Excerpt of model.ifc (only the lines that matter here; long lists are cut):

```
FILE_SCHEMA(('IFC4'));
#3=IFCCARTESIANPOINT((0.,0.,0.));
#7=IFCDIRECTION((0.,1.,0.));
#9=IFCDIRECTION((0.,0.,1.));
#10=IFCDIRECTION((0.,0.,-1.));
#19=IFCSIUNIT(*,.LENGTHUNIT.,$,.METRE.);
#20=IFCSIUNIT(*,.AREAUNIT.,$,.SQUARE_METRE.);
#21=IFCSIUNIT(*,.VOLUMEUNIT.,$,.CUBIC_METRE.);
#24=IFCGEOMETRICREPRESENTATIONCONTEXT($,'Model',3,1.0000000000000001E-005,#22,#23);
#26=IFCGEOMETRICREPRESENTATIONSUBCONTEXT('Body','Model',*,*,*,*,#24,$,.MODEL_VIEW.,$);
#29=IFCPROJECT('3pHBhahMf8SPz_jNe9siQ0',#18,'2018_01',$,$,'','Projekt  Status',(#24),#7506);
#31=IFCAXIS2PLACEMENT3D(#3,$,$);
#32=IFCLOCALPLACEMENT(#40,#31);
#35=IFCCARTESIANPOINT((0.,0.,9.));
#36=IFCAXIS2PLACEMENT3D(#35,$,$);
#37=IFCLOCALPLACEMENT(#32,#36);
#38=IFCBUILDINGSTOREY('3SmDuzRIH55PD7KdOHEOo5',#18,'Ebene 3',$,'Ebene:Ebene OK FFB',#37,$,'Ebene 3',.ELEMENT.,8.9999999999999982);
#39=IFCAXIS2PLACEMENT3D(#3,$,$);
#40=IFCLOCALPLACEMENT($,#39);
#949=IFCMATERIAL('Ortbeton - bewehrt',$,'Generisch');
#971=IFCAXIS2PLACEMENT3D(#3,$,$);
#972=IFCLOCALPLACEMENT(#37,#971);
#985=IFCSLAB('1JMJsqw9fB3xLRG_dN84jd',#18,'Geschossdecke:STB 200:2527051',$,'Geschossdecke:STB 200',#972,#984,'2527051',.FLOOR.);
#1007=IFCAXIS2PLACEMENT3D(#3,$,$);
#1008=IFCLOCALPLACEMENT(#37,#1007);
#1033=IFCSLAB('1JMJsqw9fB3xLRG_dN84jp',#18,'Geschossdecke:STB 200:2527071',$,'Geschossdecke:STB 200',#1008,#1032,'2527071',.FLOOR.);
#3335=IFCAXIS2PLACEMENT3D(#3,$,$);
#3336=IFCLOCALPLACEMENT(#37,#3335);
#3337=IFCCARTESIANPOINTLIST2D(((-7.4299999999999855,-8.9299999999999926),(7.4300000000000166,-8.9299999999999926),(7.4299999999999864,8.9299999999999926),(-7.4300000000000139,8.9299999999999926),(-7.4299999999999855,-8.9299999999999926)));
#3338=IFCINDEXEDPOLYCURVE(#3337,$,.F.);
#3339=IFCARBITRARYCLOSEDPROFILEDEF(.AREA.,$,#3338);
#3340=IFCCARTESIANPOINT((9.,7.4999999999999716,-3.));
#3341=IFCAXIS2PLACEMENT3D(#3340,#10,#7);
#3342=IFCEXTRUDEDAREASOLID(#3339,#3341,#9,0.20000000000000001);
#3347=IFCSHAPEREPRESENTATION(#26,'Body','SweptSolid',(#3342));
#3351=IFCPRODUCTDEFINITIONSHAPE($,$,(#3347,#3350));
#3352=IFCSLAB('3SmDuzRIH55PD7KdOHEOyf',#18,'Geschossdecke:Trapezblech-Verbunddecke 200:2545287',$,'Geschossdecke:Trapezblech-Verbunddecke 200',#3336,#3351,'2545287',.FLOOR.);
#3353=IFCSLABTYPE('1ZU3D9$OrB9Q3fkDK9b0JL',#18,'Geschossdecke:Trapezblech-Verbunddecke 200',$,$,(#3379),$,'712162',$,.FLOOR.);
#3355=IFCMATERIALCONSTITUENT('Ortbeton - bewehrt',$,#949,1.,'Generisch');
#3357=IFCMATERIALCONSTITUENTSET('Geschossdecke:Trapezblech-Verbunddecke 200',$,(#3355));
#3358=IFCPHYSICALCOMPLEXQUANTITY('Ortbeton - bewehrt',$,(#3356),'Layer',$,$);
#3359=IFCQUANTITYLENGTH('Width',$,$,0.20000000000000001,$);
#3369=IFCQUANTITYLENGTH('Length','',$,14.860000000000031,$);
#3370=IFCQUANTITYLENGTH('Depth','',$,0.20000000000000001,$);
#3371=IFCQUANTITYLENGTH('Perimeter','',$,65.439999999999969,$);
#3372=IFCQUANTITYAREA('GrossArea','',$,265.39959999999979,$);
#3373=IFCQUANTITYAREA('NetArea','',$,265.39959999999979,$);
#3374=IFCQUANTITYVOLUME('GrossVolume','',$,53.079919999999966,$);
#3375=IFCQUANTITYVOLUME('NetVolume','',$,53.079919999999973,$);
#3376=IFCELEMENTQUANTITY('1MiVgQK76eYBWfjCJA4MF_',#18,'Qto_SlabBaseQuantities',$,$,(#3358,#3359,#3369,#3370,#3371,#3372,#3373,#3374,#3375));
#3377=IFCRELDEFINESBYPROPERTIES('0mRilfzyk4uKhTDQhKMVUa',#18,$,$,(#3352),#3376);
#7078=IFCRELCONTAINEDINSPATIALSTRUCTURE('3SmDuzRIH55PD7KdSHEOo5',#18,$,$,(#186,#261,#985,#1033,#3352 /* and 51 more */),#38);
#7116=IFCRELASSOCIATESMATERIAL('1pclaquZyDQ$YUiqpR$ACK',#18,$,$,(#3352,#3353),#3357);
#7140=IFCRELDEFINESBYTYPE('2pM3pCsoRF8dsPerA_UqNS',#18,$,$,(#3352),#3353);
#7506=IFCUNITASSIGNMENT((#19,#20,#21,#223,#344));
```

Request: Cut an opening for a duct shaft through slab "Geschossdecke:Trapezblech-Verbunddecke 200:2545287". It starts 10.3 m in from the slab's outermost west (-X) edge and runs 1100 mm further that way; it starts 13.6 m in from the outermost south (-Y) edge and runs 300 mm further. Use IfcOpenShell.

```python
import numpy as np
import ifcopenshell
import ifcopenshell.api.feature
import ifcopenshell.api.geometry
import ifcopenshell.api.pset
import ifcopenshell.api.root
import ifcopenshell.geom
import ifcopenshell.util.element
import ifcopenshell.util.placement
import ifcopenshell.util.representation
import ifcopenshell.util.shape
import ifcopenshell.util.unit

model = ifcopenshell.open("model.ifc")
unit_scale = ifcopenshell.util.unit.calculate_unit_scale(model)
area_scale = ifcopenshell.util.unit.calculate_unit_scale(model, "AREAUNIT")
volume_scale = ifcopenshell.util.unit.calculate_unit_scale(model, "VOLUMEUNIT")
settings = ifcopenshell.geom.settings()


def volume(element):
    """Net volume in cubic metres, openings subtracted."""
    shape = ifcopenshell.geom.create_shape(settings, element)
    return ifcopenshell.util.shape.get_volume(shape.geometry)


slab = model.by_guid("3SmDuzRIH55PD7KdOHEOyf")
before = volume(slab)

# Extent in the slab's own axes, in metres. The edges named are its -X and -Y sides.
slab_shape = ifcopenshell.geom.create_shape(settings, slab)
vertices = ifcopenshell.util.shape.get_vertices(slab_shape.geometry)
x_min, y_min, bottom = vertices.min(axis=0)
top = vertices[:, 2].max()

opening = ifcopenshell.api.root.create_entity(model, ifc_class="IfcOpeningElement", name="Duct shaft opening", predefined_type="OPENING")
context = ifcopenshell.util.representation.get_context(model, "Model", "Body", "MODEL_VIEW")
width, depth = 1.1, 0.3
outline = [(0.0, 0.0), (width, 0.0), (width, depth), (0.0, depth), (0.0, 0.0)]
# Overshoot both faces by 50 mm so the cut is clean.
shape = ifcopenshell.api.geometry.add_slab_representation(
    model, context=context, depth=top - bottom + 0.1, polyline=outline
)
ifcopenshell.api.geometry.assign_representation(model, product=opening, representation=shape)

matrix = ifcopenshell.util.placement.get_local_placement(slab.ObjectPlacement)
matrix[:, 3] = matrix @ np.append(np.array([x_min + 10.3, y_min + 13.6, bottom - 0.05]) / unit_scale, 1.0)
ifcopenshell.api.geometry.edit_object_placement(model, product=opening, matrix=matrix, is_si=False)
ifcopenshell.api.feature.add_feature(model, feature=opening, element=slab)

after = volume(slab)

# Update the slab's stored quantities.
qto = model.by_id(ifcopenshell.util.element.get_pset(slab, "Qto_SlabBaseQuantities", should_inherit=False)["id"])
ifcopenshell.api.pset.edit_qto(model, qto=qto, properties={
    "NetArea": after / (top - bottom) / area_scale,
    "NetVolume": after / volume_scale,
})

print(f"slab volume {before:.3f} -> {after:.3f} m3")

model.write("model_rev.ifc")
```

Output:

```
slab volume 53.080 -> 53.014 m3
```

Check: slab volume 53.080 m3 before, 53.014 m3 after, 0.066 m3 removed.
